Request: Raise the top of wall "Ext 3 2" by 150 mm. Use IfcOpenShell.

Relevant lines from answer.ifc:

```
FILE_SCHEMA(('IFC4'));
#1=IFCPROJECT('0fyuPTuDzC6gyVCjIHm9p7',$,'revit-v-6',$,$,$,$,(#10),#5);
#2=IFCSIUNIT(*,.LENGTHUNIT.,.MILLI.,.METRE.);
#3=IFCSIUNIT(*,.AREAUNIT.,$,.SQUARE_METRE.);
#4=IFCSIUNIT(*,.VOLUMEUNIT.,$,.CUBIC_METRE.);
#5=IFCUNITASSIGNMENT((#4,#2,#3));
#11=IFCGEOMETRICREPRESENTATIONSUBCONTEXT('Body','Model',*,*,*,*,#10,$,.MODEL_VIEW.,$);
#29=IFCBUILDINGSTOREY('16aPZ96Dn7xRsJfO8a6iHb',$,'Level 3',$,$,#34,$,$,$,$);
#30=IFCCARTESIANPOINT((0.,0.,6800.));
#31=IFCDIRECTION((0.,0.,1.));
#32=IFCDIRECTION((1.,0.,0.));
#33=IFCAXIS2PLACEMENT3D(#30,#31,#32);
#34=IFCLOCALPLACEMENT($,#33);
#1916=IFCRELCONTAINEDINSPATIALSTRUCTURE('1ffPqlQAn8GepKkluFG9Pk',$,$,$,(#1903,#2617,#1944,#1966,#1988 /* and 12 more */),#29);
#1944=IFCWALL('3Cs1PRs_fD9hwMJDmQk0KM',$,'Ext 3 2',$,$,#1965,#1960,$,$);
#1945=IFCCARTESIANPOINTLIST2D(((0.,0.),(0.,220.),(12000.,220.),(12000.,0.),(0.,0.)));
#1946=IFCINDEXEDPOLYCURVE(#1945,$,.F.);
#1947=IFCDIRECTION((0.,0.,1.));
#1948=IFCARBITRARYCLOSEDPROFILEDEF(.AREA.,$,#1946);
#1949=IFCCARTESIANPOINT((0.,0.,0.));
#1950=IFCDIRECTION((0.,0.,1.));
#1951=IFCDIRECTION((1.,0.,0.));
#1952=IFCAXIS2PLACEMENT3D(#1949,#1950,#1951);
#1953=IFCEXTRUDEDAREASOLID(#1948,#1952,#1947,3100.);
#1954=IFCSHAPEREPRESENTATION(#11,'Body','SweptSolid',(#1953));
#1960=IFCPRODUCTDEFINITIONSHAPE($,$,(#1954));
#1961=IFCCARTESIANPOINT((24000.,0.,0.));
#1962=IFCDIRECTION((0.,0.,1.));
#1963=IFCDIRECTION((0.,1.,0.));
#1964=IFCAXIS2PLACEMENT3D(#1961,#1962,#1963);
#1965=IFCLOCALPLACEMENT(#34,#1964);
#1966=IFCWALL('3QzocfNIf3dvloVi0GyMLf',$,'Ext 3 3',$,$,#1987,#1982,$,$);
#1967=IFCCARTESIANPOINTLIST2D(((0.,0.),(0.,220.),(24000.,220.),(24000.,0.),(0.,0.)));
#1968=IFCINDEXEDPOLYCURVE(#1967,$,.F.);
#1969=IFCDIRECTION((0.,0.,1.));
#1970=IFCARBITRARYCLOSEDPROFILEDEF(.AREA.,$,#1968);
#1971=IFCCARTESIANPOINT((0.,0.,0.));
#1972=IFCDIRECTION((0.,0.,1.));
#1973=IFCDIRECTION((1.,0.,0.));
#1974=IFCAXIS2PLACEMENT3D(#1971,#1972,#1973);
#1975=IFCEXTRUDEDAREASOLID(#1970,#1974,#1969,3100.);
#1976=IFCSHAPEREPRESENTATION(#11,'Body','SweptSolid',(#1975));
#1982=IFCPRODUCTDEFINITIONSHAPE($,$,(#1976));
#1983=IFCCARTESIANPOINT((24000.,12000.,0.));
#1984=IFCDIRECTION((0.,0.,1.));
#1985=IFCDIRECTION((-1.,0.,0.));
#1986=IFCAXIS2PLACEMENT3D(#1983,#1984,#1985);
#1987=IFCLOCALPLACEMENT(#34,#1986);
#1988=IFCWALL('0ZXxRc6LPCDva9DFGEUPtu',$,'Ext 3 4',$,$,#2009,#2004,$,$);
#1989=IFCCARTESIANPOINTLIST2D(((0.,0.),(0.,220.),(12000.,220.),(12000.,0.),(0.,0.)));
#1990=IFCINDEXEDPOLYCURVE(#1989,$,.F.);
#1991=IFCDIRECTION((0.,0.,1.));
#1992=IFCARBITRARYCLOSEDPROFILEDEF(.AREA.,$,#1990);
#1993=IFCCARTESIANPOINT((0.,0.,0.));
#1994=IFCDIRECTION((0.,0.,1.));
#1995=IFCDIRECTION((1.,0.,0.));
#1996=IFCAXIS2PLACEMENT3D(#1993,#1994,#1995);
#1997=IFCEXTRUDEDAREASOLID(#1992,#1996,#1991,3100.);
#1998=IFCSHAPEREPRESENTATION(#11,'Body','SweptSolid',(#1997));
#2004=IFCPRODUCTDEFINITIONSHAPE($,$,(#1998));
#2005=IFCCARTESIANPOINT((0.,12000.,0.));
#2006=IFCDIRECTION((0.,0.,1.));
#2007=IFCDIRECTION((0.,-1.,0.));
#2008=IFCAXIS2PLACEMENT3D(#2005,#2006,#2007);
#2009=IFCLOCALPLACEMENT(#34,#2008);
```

```python
import ifcopenshell
import ifcopenshell.geom
import ifcopenshell.util.representation
import ifcopenshell.util.shape

model = ifcopenshell.open("answer.ifc")
settings = ifcopenshell.geom.settings()


def volume(element):
    """Net volume in cubic metres, openings subtracted."""
    shape = ifcopenshell.geom.create_shape(settings, element)
    return ifcopenshell.util.shape.get_volume(shape.geometry)


wall = model.by_id(1944)
before = volume(wall)

body = ifcopenshell.util.representation.get_representation(wall, "Model", "Body")
solid = body.Items[0]
old_height = solid.Depth
solid.Depth += 150.0
after = volume(wall)

print(f"height {old_height:g} -> {solid.Depth:g}, volume {before:.3f} -> {after:.3f} m3")

model.write("answer_edited.ifc")
```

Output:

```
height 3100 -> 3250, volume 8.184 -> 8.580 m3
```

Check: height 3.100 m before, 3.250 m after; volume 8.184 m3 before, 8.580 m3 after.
